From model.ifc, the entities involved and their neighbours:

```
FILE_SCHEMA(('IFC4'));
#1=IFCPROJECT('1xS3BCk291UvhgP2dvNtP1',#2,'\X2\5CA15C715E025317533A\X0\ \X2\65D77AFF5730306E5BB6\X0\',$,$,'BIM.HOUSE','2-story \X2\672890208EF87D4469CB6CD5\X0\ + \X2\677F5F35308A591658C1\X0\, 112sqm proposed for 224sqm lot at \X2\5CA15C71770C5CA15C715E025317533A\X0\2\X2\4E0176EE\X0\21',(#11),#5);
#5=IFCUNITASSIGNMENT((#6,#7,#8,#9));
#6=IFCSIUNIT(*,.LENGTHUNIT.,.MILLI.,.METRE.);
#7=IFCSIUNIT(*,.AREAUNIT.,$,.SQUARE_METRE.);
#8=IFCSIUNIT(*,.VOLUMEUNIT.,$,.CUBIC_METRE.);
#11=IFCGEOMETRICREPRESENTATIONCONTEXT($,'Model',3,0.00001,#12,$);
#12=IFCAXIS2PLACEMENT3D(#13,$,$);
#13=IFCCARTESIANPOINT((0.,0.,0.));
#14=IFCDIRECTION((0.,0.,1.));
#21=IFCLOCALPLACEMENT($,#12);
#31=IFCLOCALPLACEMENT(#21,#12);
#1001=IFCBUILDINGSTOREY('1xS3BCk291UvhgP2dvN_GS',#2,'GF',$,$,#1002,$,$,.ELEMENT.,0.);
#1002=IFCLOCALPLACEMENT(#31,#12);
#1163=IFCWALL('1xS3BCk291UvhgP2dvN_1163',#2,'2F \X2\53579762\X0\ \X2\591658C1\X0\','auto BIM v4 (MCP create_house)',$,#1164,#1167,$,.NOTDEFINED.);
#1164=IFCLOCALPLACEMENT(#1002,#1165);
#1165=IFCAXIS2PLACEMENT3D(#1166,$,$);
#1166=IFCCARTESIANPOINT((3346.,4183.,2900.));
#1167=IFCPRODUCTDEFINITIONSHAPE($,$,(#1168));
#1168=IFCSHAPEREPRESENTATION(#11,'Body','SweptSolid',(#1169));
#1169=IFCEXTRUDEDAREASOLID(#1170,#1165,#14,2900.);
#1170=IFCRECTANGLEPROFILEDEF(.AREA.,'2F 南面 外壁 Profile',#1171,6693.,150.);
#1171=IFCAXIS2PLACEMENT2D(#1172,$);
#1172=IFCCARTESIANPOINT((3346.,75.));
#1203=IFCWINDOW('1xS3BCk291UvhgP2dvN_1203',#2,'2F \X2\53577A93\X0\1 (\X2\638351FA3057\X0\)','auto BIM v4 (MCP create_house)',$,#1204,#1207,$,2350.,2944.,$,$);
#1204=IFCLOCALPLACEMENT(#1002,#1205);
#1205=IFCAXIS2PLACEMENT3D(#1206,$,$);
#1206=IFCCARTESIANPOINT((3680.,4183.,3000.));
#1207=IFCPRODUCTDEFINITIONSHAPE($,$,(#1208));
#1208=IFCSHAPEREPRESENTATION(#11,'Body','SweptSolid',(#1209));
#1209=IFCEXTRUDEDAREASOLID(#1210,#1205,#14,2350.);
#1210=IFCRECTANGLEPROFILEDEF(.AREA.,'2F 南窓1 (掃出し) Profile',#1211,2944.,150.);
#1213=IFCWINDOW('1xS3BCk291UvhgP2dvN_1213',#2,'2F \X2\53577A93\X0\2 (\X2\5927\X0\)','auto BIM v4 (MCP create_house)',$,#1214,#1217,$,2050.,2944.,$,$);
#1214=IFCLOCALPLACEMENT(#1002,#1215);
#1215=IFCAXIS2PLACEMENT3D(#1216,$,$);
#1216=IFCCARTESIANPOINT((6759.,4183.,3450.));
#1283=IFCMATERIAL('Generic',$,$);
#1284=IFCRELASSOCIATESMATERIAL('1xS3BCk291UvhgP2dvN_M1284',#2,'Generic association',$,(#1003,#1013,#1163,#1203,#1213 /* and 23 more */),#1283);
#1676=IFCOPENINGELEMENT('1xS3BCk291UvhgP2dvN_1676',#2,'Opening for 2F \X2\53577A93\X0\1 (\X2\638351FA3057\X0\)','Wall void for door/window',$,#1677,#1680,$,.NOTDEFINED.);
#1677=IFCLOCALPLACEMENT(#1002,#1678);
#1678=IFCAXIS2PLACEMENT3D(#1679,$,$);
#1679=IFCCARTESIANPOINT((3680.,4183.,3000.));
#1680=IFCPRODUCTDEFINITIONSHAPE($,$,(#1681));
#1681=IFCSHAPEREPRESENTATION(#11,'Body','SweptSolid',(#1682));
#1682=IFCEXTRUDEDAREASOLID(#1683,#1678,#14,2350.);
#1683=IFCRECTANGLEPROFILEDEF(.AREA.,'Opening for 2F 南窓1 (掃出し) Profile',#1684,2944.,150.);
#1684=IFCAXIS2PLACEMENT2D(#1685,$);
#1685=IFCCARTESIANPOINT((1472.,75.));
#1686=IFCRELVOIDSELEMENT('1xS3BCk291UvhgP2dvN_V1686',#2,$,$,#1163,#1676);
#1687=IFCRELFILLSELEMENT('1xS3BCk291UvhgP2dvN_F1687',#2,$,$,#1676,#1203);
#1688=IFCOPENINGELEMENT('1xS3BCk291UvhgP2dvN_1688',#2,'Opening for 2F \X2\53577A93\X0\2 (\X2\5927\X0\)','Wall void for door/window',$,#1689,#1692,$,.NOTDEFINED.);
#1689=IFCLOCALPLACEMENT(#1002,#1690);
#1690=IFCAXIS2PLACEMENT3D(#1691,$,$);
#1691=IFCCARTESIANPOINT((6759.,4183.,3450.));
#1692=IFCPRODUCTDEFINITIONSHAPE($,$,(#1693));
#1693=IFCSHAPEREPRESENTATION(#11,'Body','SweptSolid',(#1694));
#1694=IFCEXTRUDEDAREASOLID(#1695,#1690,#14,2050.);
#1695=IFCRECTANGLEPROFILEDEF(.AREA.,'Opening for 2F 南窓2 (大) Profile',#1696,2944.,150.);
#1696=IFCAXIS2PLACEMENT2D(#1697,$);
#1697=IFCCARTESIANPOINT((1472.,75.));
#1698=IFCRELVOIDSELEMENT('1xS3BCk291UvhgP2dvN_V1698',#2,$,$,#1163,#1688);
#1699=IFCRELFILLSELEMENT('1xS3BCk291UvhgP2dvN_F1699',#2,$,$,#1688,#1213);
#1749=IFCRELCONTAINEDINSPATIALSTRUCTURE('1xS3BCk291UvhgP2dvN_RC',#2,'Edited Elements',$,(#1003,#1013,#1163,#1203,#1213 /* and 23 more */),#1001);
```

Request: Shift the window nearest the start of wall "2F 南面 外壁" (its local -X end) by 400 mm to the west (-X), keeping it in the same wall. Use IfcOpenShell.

```python
import ifcopenshell
import ifcopenshell.api.geometry
import ifcopenshell.util.placement

model = ifcopenshell.open("model.ifc")

window = model.by_guid("1xS3BCk291UvhgP2dvN_1203")
opening = window.FillsVoids[0].RelatingOpeningElement
wall = opening.VoidsElements[0].RelatingBuildingElement

wall_matrix = ifcopenshell.util.placement.get_local_placement(wall.ObjectPlacement)
shift = wall_matrix[:3, 0] * -400.0
before = ifcopenshell.util.placement.get_local_placement(window.ObjectPlacement)[:3, 3].copy()

# The window is not placed relative to its opening, so move both.
for product in (opening, window):
    matrix = ifcopenshell.util.placement.get_local_placement(product.ObjectPlacement)
    matrix[:3, 3] += shift
    ifcopenshell.api.geometry.edit_object_placement(model, product=product, matrix=matrix, is_si=False)

after = ifcopenshell.util.placement.get_local_placement(window.ObjectPlacement)[:3, 3]
print("window moved by", (after - before).round(3) + 0.0)

model.write("model_edited.ifc")
```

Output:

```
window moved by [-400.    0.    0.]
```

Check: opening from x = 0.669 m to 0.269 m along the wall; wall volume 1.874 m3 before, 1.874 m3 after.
